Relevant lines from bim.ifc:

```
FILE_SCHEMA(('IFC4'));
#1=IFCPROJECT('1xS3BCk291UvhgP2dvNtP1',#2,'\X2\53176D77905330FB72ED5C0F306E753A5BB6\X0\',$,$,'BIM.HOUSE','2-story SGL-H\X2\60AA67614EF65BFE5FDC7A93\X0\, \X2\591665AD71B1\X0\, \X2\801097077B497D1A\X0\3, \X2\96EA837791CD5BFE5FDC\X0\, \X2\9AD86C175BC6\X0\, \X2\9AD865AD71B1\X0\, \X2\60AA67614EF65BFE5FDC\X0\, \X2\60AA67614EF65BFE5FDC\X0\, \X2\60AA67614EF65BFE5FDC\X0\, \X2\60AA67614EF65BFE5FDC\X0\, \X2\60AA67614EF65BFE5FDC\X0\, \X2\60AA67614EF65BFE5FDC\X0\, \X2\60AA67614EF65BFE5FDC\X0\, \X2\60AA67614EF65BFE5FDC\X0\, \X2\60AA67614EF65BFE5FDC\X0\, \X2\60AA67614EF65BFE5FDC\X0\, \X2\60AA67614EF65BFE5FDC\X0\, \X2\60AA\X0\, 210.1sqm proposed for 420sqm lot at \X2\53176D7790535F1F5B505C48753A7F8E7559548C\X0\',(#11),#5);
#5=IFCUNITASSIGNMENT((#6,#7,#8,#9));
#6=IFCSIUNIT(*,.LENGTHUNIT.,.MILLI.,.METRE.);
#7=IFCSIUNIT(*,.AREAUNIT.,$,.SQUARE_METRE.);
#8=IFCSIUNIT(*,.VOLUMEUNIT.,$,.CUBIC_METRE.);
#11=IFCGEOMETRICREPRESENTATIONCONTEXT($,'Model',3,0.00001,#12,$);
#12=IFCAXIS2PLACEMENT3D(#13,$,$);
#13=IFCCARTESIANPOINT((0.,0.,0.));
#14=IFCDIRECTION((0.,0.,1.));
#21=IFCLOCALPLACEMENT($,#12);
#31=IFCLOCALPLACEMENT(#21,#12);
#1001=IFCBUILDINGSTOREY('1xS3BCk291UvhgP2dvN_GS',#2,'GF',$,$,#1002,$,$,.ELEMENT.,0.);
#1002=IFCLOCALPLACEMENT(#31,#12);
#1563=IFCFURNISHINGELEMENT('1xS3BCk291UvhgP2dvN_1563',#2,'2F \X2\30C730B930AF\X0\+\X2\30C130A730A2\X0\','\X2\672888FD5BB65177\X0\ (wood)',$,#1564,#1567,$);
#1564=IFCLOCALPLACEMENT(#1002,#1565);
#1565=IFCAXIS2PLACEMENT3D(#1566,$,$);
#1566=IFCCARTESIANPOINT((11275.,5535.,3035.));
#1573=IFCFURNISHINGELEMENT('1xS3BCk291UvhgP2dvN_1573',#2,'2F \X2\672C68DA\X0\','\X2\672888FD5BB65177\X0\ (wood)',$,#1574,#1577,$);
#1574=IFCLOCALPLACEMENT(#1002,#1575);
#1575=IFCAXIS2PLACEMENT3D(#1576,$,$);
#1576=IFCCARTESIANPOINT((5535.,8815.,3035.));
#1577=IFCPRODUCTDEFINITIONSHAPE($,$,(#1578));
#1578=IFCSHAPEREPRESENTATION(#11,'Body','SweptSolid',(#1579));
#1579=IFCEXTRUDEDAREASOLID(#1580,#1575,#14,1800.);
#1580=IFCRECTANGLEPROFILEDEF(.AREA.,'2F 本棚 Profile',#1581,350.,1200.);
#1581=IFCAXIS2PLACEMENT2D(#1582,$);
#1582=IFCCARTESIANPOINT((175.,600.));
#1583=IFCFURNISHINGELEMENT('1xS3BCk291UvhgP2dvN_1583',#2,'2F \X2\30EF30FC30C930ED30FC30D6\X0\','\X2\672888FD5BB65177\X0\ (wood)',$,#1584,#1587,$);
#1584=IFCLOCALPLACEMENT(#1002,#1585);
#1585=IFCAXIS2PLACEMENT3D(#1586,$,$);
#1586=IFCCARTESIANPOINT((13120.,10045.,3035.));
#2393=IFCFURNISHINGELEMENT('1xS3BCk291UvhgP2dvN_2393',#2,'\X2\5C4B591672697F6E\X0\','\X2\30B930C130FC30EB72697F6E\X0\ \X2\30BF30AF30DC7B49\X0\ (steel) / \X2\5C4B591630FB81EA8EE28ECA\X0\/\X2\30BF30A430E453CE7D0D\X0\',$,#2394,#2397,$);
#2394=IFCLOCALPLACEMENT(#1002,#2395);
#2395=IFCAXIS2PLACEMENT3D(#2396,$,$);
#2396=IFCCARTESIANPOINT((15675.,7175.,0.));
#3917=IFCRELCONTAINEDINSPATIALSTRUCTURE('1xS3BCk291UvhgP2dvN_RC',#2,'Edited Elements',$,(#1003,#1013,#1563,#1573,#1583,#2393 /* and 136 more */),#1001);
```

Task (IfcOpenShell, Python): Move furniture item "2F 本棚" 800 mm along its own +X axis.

```python
import ifcopenshell
import ifcopenshell.api.geometry
import ifcopenshell.util.placement
import ifcopenshell.util.unit

model = ifcopenshell.open("bim.ifc")
unit_scale = ifcopenshell.util.unit.calculate_unit_scale(model)

item = model.by_id(1573)
matrix = ifcopenshell.util.placement.get_local_placement(item.ObjectPlacement)
matrix[:3, 3] += matrix[:3, 0] * 0.8 / unit_scale
ifcopenshell.api.geometry.edit_object_placement(model, product=item, matrix=matrix, is_si=False)

print(ifcopenshell.util.placement.get_local_placement(item.ObjectPlacement).round(3) + 0.0)

model.write("bim_v2.ifc")
```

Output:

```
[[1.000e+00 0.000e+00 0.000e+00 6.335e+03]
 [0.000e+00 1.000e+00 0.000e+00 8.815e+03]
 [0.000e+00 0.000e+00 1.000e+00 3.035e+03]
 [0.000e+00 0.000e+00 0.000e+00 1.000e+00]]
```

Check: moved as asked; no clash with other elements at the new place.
